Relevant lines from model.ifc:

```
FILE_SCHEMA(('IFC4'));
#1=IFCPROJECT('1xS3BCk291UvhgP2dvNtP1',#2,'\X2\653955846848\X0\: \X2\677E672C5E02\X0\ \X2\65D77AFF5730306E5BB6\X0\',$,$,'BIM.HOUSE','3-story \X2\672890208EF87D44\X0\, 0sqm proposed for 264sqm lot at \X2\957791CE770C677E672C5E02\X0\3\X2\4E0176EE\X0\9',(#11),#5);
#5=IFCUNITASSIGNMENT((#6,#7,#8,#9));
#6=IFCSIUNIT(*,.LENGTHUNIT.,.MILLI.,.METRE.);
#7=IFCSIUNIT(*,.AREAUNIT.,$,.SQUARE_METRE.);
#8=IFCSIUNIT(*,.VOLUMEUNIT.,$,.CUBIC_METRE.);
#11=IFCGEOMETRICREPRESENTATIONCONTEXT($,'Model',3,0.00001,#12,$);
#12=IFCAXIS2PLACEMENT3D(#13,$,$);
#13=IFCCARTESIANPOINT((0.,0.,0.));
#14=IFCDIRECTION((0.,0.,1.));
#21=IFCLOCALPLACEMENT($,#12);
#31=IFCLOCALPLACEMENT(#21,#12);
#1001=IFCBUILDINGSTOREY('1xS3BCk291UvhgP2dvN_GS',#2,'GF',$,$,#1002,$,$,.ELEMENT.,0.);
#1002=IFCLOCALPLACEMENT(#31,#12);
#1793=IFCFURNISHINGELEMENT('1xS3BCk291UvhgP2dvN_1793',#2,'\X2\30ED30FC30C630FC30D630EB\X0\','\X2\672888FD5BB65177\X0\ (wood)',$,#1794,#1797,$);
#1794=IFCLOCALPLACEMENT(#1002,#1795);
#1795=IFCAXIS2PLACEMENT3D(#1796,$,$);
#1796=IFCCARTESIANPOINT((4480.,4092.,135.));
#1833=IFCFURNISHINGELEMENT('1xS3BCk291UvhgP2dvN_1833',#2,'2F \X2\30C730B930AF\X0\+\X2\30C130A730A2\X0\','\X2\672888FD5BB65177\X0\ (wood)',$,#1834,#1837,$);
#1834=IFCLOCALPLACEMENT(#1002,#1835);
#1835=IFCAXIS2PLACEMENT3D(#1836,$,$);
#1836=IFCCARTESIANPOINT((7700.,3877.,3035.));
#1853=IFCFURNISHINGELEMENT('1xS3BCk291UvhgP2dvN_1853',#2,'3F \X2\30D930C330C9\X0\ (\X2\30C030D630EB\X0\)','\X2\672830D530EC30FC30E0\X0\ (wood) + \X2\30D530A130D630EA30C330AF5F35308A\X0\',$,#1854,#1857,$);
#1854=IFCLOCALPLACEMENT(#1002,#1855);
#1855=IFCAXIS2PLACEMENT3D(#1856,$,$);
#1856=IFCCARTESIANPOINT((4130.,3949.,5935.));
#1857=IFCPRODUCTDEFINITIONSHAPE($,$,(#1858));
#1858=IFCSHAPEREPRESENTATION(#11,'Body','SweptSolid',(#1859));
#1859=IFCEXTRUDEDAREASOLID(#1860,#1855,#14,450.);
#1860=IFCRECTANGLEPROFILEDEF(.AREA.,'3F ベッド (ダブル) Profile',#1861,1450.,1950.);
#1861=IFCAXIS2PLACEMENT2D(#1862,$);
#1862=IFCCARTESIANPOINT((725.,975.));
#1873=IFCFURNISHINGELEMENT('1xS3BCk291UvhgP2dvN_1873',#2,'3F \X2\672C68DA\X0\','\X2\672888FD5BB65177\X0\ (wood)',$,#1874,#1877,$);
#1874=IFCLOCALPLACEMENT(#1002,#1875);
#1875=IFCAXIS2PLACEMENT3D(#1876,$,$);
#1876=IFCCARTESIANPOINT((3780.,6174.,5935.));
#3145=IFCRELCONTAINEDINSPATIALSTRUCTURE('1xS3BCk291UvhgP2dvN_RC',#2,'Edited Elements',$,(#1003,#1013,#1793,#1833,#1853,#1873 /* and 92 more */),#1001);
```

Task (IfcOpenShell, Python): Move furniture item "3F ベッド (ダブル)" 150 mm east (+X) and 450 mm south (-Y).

```python
import ifcopenshell
import ifcopenshell.api.geometry
import ifcopenshell.util.placement
import ifcopenshell.util.unit

model = ifcopenshell.open("model.ifc")
unit_scale = ifcopenshell.util.unit.calculate_unit_scale(model)

item = model.by_guid("1xS3BCk291UvhgP2dvN_1853")
matrix = ifcopenshell.util.placement.get_local_placement(item.ObjectPlacement)
matrix[0, 3] += 0.15 / unit_scale
matrix[1, 3] -= 0.45 / unit_scale
ifcopenshell.api.geometry.edit_object_placement(model, product=item, matrix=matrix, is_si=False)

print(ifcopenshell.util.placement.get_local_placement(item.ObjectPlacement).round(3) + 0.0)

model.write("model_edited.ifc")
```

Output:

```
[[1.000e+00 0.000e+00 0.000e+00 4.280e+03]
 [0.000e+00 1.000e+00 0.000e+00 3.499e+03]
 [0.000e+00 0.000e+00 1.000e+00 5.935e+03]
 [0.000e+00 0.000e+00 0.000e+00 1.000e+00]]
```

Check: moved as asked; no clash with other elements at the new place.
